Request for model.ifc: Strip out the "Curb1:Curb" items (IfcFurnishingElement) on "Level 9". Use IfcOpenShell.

First a look at what the model holds.

```python
import ifcopenshell
import ifcopenshell.util.element

model = ifcopenshell.open("model.ifc")
print(model.schema)
storey = next(s for s in model.by_type("IfcBuildingStorey") if s.Name == "Level 9")
furniture = [e for e in ifcopenshell.util.element.get_decomposition(storey) if e.is_a("IfcFurnishingElement")]
seen = {}
for e in furniture:
    element_type = ifcopenshell.util.element.get_type(e)
    name = element_type.Name if element_type not in (None, e) else None
    seen[name] = seen.get(name, 0) + 1
for name, count in sorted(seen.items(), key=str):
    print(count, "x", name)
```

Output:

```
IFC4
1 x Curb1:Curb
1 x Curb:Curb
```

```python
import ifcopenshell
import ifcopenshell.api.root
import ifcopenshell.util.element

model = ifcopenshell.open("model.ifc")

storey = next(s for s in model.by_type("IfcBuildingStorey") if s.Name == "Level 9")
furniture = [e for e in ifcopenshell.util.element.get_decomposition(storey) if e.is_a("IfcFurnishingElement")]
targets = [e for e in furniture if (t := ifcopenshell.util.element.get_type(e)) not in (None, e) and t.Name == "Curb1:Curb"]

for e in targets:
    ifcopenshell.api.root.remove_product(model, product=e)
print(len(targets), "removed")

model.write("model_updated.ifc")
```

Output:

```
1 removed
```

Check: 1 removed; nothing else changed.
